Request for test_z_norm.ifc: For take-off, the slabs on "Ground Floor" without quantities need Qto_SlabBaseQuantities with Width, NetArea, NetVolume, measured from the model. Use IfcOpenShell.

First a look at what the model holds.

```python
import ifcopenshell
import ifcopenshell.util.element
import ifcopenshell.util.unit

model = ifcopenshell.open("test_z_norm.ifc")
print(model.schema)
for unit_type in ("LENGTHUNIT", "AREAUNIT", "VOLUMEUNIT"):
    print(unit_type, ifcopenshell.util.unit.calculate_unit_scale(model, unit_type))
storey = next(s for s in model.by_type("IfcBuildingStorey") if s.Name == "Ground Floor")
slabs = [e for e in ifcopenshell.util.element.get_decomposition(storey) if e.is_a("IfcSlab")]
for e in sorted(slabs, key=lambda e: e.id()):
    print(e.id(), e.is_a(), e.Name, list(ifcopenshell.util.element.get_psets(e, qtos_only=True)), sep=" | ")
```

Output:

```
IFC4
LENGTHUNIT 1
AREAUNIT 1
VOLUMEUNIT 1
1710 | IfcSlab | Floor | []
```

```python
import ifcopenshell
import ifcopenshell.api.pset
import ifcopenshell.geom
import ifcopenshell.util.element
import ifcopenshell.util.shape
import ifcopenshell.util.unit

model = ifcopenshell.open("test_z_norm.ifc")
unit_scale = ifcopenshell.util.unit.calculate_unit_scale(model)
area_scale = ifcopenshell.util.unit.calculate_unit_scale(model, "AREAUNIT")
volume_scale = ifcopenshell.util.unit.calculate_unit_scale(model, "VOLUMEUNIT")
settings = ifcopenshell.geom.settings()

storey = next(s for s in model.by_type("IfcBuildingStorey") if s.Name == "Ground Floor")
slabs = [e for e in ifcopenshell.util.element.get_decomposition(storey) if e.is_a("IfcSlab")]

for e in sorted(slabs, key=lambda e: e.id()):
    if ifcopenshell.util.element.get_psets(e, qtos_only=True, should_inherit=False):
        continue
    # Geometry comes back in metres, in the element's own axes.
    shape = ifcopenshell.geom.create_shape(settings, e)
    values = {
        "Width": ifcopenshell.util.shape.get_z(shape.geometry) / unit_scale,
        "NetArea": ifcopenshell.util.shape.get_footprint_area(shape.geometry) / area_scale,
        "NetVolume": ifcopenshell.util.shape.get_volume(shape.geometry) / volume_scale,
    }
    qto = ifcopenshell.api.pset.add_qto(model, product=e, name="Qto_SlabBaseQuantities")
    ifcopenshell.api.pset.edit_qto(model, qto=qto, properties=values)
    print(e.id(), {k: round(v, 3) for k, v in values.items()})

model.write("test_z_norm_v2.ifc")
```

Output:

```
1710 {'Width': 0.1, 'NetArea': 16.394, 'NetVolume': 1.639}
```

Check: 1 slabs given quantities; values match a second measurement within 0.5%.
